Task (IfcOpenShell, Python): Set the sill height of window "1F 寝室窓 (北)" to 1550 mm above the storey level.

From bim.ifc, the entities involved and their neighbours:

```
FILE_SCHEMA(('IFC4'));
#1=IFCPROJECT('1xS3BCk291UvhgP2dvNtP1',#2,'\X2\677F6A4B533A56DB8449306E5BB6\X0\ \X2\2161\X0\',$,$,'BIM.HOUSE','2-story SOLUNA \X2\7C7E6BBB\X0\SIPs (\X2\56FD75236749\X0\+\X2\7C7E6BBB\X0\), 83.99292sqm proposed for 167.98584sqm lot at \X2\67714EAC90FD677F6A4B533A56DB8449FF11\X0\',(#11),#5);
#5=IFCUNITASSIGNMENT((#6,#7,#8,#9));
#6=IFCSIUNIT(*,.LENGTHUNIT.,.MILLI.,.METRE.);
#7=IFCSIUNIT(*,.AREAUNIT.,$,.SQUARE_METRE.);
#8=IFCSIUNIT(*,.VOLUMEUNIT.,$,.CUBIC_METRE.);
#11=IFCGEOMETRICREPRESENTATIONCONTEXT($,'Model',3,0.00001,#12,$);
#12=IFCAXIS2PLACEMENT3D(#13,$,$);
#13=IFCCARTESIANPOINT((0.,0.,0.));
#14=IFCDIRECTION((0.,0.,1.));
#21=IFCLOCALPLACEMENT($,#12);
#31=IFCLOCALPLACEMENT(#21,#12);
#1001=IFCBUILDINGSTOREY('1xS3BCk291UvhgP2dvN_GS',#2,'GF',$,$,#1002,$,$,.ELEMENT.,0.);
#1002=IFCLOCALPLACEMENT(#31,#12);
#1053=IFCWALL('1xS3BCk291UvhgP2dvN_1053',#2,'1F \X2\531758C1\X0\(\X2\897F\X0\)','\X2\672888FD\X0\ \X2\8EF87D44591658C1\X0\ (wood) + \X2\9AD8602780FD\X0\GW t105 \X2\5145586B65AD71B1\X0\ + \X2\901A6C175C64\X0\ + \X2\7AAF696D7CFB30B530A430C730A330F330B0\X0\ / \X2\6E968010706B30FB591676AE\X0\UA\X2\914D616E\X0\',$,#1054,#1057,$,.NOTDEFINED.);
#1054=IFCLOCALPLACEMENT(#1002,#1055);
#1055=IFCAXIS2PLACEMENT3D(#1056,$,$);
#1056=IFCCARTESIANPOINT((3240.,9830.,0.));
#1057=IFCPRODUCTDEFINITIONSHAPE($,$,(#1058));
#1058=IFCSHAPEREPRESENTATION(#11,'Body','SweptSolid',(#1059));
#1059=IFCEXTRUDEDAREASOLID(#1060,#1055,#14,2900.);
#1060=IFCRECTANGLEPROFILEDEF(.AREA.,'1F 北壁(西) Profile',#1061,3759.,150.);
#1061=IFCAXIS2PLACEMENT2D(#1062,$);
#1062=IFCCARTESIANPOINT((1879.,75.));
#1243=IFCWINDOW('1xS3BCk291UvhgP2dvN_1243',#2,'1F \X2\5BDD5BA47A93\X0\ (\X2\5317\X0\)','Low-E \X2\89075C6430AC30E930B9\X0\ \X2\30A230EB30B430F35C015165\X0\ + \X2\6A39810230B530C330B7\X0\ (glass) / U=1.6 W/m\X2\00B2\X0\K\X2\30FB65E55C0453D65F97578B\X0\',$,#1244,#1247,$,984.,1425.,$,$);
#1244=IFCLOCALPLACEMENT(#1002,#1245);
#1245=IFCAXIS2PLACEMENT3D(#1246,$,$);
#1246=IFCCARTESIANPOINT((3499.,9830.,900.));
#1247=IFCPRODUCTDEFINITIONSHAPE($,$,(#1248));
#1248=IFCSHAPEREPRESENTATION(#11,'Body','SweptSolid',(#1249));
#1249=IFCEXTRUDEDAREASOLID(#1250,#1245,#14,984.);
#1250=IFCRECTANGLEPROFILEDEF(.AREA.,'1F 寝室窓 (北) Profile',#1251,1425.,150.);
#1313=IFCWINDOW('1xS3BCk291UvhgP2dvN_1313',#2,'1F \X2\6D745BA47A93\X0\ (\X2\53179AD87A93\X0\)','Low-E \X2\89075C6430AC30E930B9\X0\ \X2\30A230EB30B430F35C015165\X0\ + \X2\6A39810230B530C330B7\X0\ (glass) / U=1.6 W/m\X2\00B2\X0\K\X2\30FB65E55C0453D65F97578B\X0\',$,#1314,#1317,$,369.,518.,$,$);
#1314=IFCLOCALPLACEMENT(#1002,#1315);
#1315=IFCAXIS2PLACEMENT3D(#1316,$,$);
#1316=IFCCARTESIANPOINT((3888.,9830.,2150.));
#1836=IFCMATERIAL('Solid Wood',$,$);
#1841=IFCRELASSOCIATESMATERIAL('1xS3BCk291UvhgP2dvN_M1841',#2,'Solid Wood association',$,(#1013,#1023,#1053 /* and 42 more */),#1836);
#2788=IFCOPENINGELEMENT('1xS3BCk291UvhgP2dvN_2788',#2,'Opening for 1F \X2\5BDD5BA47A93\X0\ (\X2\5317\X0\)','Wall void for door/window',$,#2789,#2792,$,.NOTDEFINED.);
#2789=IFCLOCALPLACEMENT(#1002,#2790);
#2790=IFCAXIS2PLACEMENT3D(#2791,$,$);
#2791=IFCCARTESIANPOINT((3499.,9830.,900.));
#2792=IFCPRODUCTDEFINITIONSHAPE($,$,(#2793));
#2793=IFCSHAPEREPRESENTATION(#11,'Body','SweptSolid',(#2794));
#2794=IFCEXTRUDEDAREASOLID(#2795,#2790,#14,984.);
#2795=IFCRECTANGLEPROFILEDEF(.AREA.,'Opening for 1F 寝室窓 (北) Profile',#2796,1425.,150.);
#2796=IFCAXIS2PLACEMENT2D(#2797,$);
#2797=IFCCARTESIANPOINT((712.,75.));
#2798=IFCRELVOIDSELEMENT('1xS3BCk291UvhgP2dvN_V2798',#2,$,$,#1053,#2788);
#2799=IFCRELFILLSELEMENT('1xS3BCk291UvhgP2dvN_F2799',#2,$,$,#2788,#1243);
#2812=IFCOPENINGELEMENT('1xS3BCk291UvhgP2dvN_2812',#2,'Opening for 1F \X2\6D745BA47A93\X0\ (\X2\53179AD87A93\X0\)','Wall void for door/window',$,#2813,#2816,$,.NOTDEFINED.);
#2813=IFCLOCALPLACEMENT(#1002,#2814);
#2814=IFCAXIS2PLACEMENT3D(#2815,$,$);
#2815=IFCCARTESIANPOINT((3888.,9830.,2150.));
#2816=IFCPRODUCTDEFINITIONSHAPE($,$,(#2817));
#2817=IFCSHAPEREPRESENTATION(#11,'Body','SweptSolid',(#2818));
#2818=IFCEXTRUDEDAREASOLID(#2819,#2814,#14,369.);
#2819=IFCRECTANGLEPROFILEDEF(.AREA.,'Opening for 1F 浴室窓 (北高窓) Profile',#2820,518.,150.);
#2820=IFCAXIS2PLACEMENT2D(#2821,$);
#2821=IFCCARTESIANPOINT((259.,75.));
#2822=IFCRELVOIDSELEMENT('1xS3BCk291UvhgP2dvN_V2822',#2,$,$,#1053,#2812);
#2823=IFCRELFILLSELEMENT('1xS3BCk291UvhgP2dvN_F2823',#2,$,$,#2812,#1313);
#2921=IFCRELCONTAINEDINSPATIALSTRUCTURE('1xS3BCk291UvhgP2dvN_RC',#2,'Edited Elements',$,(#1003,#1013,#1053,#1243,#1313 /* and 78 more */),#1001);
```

```python
import numpy as np
import ifcopenshell
import ifcopenshell.api.geometry
import ifcopenshell.geom
import ifcopenshell.util.element
import ifcopenshell.util.placement
import ifcopenshell.util.shape
import ifcopenshell.util.unit

model = ifcopenshell.open("bim.ifc")
unit_scale = ifcopenshell.util.unit.calculate_unit_scale(model)

window = model.by_id(1243)
opening = window.FillsVoids[0].RelatingOpeningElement
storey = ifcopenshell.util.element.get_container(window, ifc_class="IfcBuildingStorey")
level = ifcopenshell.util.placement.get_local_placement(storey.ObjectPlacement)[2, 3]

# The opening's origin need not be at the sill, so measure its lowest point.
shape = ifcopenshell.geom.create_shape(ifcopenshell.geom.settings(), opening)
bottom = ifcopenshell.util.shape.get_shape_bottom_elevation(shape, shape.geometry) / unit_scale
dz = level + 1550.0 - bottom

shift = np.array([0.0, 0.0, dz])
# The window is not placed relative to its opening, so move both.
for product in (opening, window):
    matrix = ifcopenshell.util.placement.get_local_placement(product.ObjectPlacement)
    matrix[:3, 3] += shift
    ifcopenshell.api.geometry.edit_object_placement(model, product=product, matrix=matrix, is_si=False)

print(f"moved by {dz * unit_scale:+.3f} m")

model.write("bim_updated.ifc")
```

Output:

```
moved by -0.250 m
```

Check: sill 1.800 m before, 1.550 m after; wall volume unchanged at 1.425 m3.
